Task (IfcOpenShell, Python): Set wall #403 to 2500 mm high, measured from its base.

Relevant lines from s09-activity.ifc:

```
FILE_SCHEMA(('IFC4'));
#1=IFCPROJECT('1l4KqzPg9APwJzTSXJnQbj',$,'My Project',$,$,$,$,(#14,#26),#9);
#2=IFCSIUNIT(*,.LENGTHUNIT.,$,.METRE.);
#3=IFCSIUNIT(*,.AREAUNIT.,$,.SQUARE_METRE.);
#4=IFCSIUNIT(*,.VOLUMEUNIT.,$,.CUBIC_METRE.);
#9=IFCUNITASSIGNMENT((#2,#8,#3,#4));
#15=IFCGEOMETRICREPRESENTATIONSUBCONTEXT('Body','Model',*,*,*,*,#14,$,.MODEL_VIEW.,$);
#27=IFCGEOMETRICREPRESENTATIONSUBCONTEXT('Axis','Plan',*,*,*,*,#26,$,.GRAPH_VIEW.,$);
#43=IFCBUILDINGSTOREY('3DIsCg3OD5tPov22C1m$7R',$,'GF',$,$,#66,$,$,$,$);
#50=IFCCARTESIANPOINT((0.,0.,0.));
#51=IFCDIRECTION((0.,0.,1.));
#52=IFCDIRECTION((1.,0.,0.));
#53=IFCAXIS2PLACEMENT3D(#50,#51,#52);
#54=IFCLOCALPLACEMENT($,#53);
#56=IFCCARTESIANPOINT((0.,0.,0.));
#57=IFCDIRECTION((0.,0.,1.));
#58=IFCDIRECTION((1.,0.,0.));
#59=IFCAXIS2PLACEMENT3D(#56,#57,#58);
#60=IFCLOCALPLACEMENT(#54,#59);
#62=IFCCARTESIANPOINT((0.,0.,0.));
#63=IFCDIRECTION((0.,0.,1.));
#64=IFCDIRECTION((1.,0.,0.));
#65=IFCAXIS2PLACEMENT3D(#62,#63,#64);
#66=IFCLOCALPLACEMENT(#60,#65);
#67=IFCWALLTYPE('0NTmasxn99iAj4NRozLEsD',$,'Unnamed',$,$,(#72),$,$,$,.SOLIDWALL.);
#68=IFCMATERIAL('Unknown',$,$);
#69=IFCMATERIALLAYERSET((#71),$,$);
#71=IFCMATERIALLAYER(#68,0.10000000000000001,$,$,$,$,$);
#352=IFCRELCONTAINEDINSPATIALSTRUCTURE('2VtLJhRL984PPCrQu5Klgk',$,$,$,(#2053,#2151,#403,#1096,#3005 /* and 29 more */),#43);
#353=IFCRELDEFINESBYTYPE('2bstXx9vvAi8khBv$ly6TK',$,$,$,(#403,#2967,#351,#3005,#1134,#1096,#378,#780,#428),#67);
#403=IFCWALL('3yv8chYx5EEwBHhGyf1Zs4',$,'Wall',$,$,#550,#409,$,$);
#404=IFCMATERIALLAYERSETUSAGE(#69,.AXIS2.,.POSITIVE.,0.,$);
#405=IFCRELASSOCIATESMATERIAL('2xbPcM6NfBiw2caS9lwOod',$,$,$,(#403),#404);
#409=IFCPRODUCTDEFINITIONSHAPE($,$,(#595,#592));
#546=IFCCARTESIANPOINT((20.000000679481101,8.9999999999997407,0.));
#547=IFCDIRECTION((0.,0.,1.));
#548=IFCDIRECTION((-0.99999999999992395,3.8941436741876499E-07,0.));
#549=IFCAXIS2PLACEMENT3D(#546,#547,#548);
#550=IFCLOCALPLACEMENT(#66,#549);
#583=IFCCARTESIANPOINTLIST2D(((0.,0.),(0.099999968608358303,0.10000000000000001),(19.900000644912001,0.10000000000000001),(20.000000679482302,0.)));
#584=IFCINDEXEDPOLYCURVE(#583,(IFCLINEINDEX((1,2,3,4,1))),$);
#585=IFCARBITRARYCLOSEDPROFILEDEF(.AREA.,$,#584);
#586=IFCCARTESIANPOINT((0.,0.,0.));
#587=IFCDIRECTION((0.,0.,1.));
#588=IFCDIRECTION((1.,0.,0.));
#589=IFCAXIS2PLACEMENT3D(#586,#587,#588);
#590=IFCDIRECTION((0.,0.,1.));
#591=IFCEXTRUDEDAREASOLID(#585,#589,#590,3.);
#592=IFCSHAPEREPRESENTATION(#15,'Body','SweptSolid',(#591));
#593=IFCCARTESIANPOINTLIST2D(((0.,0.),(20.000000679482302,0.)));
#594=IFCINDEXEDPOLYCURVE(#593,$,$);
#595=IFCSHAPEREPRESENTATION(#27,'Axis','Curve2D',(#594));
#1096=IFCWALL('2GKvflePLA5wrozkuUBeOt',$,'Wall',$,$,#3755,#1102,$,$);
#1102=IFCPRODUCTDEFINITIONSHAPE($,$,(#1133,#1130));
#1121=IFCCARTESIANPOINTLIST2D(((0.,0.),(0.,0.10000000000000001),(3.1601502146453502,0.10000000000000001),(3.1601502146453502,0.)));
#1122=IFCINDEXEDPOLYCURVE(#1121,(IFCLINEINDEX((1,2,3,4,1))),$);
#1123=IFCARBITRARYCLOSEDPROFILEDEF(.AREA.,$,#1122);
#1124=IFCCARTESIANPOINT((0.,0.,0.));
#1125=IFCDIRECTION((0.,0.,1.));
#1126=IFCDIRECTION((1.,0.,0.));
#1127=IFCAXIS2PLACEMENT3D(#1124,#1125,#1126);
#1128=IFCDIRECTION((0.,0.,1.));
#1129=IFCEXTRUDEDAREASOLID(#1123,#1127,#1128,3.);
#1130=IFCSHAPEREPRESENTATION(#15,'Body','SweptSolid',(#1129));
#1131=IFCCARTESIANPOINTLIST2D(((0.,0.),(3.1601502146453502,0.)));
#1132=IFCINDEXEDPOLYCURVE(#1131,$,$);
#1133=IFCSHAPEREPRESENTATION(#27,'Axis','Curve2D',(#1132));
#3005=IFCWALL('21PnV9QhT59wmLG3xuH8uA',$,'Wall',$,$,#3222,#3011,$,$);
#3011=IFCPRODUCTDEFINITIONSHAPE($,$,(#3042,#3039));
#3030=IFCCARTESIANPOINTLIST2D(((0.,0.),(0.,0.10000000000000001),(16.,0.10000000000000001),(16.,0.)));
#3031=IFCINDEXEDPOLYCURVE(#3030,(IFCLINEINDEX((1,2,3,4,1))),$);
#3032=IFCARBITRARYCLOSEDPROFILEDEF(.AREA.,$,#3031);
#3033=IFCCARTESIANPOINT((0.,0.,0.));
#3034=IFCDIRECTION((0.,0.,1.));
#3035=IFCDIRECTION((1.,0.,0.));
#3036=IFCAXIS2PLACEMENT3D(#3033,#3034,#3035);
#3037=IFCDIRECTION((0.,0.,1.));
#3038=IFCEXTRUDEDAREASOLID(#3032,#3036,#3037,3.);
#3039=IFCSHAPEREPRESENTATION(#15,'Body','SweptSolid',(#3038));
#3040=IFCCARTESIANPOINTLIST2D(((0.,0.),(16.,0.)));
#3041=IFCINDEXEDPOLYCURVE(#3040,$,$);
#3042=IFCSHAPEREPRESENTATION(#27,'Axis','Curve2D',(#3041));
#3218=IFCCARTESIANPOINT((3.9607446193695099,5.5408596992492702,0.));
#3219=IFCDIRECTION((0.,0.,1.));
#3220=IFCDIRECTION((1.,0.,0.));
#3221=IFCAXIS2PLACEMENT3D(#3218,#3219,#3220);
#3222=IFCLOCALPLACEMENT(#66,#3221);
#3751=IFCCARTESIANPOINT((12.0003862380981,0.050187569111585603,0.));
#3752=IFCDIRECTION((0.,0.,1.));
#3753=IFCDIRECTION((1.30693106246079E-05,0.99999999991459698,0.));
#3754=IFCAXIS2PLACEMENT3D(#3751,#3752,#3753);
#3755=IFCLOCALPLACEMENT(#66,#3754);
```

```python
import ifcopenshell
import ifcopenshell.geom
import ifcopenshell.util.representation
import ifcopenshell.util.shape
import ifcopenshell.util.unit

model = ifcopenshell.open("s09-activity.ifc")
unit_scale = ifcopenshell.util.unit.calculate_unit_scale(model)
settings = ifcopenshell.geom.settings()


def volume(element):
    """Net volume in cubic metres, openings subtracted."""
    shape = ifcopenshell.geom.create_shape(settings, element)
    return ifcopenshell.util.shape.get_volume(shape.geometry)


wall = model.by_guid("3yv8chYx5EEwBHhGyf1Zs4")
before = volume(wall)

body = ifcopenshell.util.representation.get_representation(wall, "Model", "Body")
solid = body.Items[0]
old_height = solid.Depth
solid.Depth = 2.5 / unit_scale
after = volume(wall)

print(f"height {old_height:g} -> {solid.Depth:g}, volume {before:.3f} -> {after:.3f} m3")

model.write("s09-activity_edited.ifc")
```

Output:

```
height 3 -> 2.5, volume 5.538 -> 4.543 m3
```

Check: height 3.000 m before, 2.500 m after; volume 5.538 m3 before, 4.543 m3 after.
